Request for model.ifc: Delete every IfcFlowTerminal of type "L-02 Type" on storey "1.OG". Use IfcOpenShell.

First a look at what the model holds.

```python
import ifcopenshell
import ifcopenshell.util.element

model = ifcopenshell.open("model.ifc")
print(model.schema)
storey = next(s for s in model.by_type("IfcBuildingStorey") if s.Name == "1.OG")
terminals = [e for e in ifcopenshell.util.element.get_decomposition(storey) if e.is_a("IfcFlowTerminal")]
seen = {}
for e in terminals:
    element_type = ifcopenshell.util.element.get_type(e)
    name = element_type.Name if element_type not in (None, e) else None
    seen[name] = seen.get(name, 0) + 1
for name, count in sorted(seen.items(), key=str):
    print(count, "x", name)
```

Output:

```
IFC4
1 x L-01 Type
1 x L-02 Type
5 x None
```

```python
import ifcopenshell
import ifcopenshell.api.root
import ifcopenshell.util.element

model = ifcopenshell.open("model.ifc")

storey = next(s for s in model.by_type("IfcBuildingStorey") if s.Name == "1.OG")
terminals = [e for e in ifcopenshell.util.element.get_decomposition(storey) if e.is_a("IfcFlowTerminal")]
targets = [e for e in terminals if (t := ifcopenshell.util.element.get_type(e)) not in (None, e) and t.Name == "L-02 Type"]

for e in targets:
    ifcopenshell.api.root.remove_product(model, product=e)
print(len(targets), "removed")

model.write("model-out.ifc")
```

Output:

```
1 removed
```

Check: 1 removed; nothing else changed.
